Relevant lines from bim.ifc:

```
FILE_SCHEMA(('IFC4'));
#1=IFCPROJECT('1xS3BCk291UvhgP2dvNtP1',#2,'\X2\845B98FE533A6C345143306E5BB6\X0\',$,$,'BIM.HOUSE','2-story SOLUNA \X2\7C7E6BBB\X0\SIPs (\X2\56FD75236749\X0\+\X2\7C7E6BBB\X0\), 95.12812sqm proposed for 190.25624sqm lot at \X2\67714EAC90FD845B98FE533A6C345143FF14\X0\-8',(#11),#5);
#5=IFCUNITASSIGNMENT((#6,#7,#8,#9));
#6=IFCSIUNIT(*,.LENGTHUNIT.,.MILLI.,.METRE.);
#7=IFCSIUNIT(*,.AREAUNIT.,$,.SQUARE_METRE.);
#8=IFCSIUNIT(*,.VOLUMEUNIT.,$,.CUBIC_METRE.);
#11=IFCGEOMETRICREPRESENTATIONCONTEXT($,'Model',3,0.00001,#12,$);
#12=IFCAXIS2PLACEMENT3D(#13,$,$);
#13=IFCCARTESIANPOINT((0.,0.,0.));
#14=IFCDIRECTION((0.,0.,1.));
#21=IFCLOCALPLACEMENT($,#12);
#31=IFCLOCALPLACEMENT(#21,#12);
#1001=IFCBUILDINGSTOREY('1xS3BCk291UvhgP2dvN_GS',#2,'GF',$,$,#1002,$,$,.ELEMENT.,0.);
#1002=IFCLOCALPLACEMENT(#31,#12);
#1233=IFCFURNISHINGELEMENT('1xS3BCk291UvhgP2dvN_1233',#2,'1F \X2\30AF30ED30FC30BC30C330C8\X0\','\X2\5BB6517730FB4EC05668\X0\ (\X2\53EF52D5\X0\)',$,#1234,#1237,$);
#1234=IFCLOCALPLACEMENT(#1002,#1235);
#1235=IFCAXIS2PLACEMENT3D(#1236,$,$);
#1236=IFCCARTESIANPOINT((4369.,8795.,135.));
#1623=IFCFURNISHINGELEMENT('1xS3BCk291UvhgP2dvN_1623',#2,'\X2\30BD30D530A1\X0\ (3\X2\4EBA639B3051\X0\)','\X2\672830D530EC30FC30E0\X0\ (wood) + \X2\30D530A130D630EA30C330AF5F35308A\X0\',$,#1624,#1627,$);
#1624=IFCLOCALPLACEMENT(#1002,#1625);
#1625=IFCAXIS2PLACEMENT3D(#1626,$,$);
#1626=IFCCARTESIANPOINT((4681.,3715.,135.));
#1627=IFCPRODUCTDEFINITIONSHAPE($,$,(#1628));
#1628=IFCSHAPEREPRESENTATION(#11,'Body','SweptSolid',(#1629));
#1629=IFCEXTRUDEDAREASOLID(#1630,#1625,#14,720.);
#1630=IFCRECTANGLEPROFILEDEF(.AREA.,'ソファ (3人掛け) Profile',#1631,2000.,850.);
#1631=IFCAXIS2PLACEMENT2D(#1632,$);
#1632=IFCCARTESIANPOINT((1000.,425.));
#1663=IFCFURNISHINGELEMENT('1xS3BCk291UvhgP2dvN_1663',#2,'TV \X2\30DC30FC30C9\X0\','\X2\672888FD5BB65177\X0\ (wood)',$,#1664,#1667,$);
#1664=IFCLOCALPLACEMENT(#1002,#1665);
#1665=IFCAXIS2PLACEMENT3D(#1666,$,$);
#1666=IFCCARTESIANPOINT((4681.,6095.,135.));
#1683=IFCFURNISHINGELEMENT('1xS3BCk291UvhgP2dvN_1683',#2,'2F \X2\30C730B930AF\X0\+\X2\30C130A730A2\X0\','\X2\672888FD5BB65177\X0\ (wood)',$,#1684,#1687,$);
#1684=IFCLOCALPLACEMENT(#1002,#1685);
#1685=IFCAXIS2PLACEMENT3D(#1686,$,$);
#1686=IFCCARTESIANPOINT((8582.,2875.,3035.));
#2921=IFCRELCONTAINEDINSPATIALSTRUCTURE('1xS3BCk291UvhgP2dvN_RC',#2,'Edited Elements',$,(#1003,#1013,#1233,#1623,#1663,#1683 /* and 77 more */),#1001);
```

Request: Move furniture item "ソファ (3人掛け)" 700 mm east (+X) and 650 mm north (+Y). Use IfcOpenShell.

```python
import ifcopenshell
import ifcopenshell.api.geometry
import ifcopenshell.util.placement

model = ifcopenshell.open("bim.ifc")

item = model.by_guid("1xS3BCk291UvhgP2dvN_1623")
matrix = ifcopenshell.util.placement.get_local_placement(item.ObjectPlacement)
matrix[0, 3] += 700.0
matrix[1, 3] += 650.0
ifcopenshell.api.geometry.edit_object_placement(model, product=item, matrix=matrix, is_si=False)

print(ifcopenshell.util.placement.get_local_placement(item.ObjectPlacement).round(3) + 0.0)

model.write("bim_updated.ifc")
```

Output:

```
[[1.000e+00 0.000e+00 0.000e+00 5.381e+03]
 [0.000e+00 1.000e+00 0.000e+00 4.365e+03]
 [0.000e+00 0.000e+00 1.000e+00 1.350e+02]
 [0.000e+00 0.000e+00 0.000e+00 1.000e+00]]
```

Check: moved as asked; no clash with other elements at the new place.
